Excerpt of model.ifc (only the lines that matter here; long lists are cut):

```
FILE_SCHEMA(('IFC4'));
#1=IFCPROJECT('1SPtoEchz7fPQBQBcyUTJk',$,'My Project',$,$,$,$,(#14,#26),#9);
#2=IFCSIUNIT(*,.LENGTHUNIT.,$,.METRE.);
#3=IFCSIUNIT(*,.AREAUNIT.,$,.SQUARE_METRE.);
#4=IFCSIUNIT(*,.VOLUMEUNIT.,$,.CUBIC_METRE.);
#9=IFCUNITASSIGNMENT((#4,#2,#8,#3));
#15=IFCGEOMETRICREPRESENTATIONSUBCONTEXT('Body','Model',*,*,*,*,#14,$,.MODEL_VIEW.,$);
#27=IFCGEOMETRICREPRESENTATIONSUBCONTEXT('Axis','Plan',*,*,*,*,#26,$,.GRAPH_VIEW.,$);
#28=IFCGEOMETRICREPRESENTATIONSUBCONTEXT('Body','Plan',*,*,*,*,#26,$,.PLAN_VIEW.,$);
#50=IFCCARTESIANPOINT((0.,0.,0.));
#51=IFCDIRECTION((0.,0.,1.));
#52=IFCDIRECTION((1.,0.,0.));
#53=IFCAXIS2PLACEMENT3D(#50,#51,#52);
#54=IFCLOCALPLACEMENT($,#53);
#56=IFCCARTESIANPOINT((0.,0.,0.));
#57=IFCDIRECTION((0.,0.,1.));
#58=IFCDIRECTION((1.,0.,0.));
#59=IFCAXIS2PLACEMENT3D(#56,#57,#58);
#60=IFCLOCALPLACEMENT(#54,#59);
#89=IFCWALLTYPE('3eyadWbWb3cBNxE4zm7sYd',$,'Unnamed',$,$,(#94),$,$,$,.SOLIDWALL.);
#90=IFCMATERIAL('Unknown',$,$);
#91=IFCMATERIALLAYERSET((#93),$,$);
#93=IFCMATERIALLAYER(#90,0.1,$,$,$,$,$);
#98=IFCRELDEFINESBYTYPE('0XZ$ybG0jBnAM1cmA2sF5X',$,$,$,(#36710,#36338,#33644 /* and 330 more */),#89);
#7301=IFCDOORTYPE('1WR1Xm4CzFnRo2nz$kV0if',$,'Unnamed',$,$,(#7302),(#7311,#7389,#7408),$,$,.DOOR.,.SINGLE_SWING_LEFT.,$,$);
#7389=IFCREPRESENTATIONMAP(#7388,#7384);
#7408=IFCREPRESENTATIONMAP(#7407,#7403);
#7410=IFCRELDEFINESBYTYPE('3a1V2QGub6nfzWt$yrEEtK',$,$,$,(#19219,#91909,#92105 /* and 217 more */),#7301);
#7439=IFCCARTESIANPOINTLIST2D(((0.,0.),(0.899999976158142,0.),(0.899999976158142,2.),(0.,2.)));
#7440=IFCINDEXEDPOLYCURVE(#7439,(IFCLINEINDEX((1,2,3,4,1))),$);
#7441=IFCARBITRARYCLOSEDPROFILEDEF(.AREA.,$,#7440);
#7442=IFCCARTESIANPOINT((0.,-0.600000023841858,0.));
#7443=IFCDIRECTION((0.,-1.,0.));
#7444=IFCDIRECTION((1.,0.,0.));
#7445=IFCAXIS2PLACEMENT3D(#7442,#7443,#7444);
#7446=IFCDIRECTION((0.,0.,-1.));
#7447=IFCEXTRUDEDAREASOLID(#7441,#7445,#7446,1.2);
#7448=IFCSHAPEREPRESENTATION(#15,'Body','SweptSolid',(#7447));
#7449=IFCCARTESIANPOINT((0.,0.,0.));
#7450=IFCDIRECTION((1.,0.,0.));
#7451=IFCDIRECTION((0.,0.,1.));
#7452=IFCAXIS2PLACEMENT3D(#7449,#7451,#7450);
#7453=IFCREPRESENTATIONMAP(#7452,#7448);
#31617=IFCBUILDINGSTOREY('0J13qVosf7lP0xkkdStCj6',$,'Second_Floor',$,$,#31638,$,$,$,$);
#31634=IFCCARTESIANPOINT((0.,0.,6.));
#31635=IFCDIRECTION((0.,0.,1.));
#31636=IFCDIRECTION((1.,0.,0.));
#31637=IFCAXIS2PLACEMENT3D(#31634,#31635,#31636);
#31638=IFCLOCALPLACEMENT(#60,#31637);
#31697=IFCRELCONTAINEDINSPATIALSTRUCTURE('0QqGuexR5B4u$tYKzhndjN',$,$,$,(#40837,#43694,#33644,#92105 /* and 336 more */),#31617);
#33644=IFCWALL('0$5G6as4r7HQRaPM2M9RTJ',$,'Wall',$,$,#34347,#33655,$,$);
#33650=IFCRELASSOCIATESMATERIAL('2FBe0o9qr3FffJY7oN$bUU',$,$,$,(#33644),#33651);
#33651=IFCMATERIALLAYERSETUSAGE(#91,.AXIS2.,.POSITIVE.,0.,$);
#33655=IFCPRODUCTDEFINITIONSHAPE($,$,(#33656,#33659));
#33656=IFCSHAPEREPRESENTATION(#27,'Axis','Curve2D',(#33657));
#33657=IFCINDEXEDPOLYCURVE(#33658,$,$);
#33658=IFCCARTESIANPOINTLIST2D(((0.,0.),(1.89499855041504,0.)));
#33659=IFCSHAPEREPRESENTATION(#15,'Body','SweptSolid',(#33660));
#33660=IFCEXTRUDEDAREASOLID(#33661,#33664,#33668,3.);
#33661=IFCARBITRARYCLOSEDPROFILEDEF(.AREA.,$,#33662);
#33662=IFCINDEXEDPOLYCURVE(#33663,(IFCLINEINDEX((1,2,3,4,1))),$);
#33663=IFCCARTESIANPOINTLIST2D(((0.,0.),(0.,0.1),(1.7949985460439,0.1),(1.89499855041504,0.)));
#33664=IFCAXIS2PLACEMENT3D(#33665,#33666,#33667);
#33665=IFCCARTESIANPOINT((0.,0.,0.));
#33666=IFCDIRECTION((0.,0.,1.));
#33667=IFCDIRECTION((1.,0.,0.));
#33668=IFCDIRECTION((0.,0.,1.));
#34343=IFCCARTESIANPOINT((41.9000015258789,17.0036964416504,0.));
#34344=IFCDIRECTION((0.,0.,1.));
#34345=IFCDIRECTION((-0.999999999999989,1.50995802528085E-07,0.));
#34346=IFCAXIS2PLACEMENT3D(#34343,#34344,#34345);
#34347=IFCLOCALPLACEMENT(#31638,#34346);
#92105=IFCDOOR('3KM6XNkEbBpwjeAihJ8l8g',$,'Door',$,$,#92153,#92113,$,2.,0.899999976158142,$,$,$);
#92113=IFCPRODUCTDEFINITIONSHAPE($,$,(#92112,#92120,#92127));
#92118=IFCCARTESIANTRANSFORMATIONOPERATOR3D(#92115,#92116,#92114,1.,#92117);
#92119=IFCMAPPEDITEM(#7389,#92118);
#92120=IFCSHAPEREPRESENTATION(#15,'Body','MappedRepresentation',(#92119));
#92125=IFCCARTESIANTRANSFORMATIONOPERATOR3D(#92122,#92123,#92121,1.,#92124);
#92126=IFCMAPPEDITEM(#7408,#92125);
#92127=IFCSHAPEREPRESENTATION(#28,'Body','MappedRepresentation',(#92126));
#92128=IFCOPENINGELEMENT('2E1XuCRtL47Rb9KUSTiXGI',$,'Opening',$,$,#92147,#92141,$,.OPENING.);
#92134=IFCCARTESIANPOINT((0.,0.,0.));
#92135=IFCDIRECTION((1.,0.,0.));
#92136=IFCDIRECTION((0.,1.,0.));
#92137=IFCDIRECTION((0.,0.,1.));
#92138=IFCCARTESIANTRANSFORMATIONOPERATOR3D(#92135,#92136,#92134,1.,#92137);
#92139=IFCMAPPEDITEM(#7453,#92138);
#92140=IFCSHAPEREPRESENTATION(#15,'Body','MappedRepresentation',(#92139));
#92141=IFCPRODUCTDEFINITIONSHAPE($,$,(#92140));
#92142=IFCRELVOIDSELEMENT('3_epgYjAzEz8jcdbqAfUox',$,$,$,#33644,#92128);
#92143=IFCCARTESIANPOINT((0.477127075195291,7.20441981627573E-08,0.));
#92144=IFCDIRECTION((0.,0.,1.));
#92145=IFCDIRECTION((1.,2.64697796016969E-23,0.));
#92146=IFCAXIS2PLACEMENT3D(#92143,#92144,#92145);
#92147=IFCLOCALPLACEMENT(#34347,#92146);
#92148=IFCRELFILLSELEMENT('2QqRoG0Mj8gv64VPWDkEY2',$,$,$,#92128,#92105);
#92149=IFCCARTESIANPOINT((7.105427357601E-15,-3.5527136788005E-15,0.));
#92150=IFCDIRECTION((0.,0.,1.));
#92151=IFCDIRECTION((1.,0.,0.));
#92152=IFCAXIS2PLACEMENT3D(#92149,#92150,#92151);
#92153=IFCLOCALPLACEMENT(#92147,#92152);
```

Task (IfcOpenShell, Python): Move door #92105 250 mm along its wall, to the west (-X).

```python
import ifcopenshell
import ifcopenshell.api.geometry
import ifcopenshell.util.placement

model = ifcopenshell.open("model.ifc")

door = model.by_guid("3KM6XNkEbBpwjeAihJ8l8g")
opening = door.FillsVoids[0].RelatingOpeningElement
wall = opening.VoidsElements[0].RelatingBuildingElement

wall_matrix = ifcopenshell.util.placement.get_local_placement(wall.ObjectPlacement)
shift = wall_matrix[:3, 0] * 0.25
before = ifcopenshell.util.placement.get_local_placement(door.ObjectPlacement)[:3, 3].copy()

# The door is placed relative to its opening, so it follows when the opening moves.
matrix = ifcopenshell.util.placement.get_local_placement(opening.ObjectPlacement)
matrix[:3, 3] += shift
ifcopenshell.api.geometry.edit_object_placement(
    model, product=opening, matrix=matrix, is_si=False, should_transform_children=True
)

after = ifcopenshell.util.placement.get_local_placement(door.ObjectPlacement)[:3, 3]
print("door moved by", (after - before).round(3) + 0.0)

model.write("model_edited.ifc")
```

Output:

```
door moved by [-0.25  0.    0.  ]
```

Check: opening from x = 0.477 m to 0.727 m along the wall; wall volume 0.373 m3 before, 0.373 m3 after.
